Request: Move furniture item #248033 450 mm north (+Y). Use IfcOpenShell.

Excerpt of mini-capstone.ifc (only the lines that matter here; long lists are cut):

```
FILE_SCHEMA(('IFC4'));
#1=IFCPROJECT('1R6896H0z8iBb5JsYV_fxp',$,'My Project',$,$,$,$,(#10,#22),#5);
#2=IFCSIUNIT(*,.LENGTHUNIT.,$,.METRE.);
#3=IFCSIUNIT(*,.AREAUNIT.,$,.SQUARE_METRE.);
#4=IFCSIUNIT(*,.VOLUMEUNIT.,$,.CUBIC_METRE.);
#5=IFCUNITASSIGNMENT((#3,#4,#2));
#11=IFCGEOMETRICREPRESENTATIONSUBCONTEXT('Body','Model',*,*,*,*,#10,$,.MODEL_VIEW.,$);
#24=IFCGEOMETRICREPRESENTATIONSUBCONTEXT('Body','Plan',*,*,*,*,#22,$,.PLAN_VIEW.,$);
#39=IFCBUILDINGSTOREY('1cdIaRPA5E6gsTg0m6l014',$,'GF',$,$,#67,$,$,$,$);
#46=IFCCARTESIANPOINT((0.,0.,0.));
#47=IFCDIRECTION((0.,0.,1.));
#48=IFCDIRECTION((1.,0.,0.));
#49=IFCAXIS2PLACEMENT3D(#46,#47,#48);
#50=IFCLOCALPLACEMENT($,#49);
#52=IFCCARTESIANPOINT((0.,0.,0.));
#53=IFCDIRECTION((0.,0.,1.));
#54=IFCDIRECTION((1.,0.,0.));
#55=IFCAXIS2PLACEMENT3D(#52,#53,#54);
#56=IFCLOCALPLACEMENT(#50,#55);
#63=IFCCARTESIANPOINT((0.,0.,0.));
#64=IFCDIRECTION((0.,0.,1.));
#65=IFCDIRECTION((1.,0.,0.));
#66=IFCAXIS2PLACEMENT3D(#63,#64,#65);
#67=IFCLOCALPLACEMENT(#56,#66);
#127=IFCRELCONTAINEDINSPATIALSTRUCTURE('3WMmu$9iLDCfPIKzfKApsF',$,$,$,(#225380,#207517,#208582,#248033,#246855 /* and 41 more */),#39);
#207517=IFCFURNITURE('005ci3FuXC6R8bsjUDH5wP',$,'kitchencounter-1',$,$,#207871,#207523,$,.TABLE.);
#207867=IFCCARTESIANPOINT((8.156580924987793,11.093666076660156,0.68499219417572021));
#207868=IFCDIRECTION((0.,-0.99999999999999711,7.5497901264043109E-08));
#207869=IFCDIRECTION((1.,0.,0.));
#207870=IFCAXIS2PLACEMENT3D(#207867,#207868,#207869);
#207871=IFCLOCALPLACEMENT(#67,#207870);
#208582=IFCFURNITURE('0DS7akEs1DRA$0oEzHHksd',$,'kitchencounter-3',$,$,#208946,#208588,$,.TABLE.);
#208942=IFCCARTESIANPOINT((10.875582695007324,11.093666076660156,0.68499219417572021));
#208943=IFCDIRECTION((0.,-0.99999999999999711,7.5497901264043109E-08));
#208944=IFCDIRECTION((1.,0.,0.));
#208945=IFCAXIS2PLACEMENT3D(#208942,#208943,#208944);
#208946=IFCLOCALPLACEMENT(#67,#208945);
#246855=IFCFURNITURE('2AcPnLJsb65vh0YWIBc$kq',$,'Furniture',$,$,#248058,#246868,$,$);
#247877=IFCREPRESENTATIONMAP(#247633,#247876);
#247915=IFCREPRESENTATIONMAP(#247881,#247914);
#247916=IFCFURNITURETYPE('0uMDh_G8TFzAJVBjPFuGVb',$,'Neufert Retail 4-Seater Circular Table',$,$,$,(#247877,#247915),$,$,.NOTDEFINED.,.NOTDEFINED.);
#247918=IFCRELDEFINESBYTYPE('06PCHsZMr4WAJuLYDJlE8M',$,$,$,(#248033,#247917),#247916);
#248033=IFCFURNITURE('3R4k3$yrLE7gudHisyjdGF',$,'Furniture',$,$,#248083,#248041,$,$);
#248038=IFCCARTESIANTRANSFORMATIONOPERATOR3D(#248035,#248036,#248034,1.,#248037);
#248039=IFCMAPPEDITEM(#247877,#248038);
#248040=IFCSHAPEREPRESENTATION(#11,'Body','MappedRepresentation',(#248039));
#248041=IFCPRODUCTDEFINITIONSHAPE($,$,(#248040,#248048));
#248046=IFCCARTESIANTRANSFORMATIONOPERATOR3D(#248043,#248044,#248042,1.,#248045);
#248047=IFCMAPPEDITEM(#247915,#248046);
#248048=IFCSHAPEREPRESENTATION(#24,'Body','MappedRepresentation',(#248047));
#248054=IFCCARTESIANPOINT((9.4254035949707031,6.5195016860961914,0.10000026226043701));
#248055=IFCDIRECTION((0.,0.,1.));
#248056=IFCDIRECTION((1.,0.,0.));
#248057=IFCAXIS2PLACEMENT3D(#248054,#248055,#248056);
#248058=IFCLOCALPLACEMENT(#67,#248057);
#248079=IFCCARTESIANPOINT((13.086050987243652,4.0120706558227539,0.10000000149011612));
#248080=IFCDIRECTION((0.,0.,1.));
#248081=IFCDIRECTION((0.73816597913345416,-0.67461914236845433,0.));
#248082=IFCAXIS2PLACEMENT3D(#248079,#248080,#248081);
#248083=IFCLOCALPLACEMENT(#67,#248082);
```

```python
import ifcopenshell
import ifcopenshell.api.geometry
import ifcopenshell.util.placement

model = ifcopenshell.open("mini-capstone.ifc")

item = model.by_guid("3R4k3$yrLE7gudHisyjdGF")
matrix = ifcopenshell.util.placement.get_local_placement(item.ObjectPlacement)
matrix[1, 3] += 0.45
ifcopenshell.api.geometry.edit_object_placement(model, product=item, matrix=matrix, is_si=False)

print(ifcopenshell.util.placement.get_local_placement(item.ObjectPlacement).round(3) + 0.0)

model.write("mini-capstone-out.ifc")
```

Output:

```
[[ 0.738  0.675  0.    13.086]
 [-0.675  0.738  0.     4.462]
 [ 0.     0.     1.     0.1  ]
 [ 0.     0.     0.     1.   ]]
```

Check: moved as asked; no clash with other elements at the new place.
